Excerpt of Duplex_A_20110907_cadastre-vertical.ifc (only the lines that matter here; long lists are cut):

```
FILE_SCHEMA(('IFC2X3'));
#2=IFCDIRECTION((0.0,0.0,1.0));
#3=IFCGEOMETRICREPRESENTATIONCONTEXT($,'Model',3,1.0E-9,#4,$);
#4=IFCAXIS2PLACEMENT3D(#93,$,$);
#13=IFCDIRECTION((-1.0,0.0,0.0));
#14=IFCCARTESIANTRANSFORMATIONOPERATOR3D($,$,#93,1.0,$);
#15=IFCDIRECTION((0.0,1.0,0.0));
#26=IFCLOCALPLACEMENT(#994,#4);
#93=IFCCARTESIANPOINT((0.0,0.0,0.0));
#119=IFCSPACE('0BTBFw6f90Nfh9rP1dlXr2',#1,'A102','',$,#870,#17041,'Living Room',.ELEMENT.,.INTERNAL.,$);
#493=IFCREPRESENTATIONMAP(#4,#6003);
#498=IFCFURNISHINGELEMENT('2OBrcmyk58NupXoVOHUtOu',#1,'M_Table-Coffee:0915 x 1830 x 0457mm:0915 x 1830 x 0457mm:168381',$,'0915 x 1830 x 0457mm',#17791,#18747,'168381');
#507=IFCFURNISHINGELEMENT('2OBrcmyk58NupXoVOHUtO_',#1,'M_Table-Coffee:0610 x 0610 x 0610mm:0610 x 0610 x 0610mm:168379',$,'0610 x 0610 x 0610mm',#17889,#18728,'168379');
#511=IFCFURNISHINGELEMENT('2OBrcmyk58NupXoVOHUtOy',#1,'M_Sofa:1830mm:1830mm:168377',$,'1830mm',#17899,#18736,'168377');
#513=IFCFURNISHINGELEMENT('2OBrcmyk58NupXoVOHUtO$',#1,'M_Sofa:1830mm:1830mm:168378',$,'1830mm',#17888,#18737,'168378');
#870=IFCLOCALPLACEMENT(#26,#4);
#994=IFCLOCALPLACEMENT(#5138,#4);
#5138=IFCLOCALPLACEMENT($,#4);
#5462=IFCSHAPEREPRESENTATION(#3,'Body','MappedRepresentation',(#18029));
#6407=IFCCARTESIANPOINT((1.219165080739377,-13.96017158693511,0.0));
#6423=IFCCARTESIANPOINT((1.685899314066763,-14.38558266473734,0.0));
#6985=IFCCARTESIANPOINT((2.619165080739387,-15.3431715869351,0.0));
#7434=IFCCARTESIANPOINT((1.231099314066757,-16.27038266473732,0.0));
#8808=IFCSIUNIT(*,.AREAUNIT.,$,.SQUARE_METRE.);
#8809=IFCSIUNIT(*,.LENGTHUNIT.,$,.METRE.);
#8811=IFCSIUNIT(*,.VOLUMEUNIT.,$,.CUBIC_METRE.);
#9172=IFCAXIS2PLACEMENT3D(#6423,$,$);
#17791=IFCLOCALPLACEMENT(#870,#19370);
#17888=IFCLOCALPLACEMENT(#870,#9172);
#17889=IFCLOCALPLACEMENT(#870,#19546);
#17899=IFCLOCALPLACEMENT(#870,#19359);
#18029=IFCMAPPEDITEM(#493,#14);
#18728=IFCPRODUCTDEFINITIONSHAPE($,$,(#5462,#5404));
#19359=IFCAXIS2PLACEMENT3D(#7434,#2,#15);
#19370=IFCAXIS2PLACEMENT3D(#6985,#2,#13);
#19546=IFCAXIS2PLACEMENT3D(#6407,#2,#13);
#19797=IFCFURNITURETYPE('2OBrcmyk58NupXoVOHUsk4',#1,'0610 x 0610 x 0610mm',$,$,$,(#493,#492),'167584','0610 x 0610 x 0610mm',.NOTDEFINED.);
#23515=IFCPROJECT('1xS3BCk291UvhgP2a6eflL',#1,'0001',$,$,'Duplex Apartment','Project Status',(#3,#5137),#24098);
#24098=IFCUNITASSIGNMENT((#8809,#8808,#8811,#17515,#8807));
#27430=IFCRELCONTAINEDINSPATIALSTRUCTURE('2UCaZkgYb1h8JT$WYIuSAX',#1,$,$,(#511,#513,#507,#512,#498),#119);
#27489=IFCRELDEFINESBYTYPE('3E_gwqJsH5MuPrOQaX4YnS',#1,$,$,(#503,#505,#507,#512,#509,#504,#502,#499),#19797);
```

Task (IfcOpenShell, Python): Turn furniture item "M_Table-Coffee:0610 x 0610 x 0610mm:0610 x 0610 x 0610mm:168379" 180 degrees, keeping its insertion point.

```python
import ifcopenshell
import ifcopenshell.api.geometry
import ifcopenshell.util.placement

model = ifcopenshell.open("Duplex_A_20110907_cadastre-vertical.ifc")

item = model.by_guid("2OBrcmyk58NupXoVOHUtO_")
matrix = ifcopenshell.util.placement.get_local_placement(item.ObjectPlacement)
matrix = matrix @ ifcopenshell.util.placement.rotation(180, "Z")
ifcopenshell.api.geometry.edit_object_placement(model, product=item, matrix=matrix, is_si=False)

print(ifcopenshell.util.placement.get_local_placement(item.ObjectPlacement).round(3) + 0.0)

model.write("Duplex_A_20110907_cadastre-vertical_updated.ifc")
```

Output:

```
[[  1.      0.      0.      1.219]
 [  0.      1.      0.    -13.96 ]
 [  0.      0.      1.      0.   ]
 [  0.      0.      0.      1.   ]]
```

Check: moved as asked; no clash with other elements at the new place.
